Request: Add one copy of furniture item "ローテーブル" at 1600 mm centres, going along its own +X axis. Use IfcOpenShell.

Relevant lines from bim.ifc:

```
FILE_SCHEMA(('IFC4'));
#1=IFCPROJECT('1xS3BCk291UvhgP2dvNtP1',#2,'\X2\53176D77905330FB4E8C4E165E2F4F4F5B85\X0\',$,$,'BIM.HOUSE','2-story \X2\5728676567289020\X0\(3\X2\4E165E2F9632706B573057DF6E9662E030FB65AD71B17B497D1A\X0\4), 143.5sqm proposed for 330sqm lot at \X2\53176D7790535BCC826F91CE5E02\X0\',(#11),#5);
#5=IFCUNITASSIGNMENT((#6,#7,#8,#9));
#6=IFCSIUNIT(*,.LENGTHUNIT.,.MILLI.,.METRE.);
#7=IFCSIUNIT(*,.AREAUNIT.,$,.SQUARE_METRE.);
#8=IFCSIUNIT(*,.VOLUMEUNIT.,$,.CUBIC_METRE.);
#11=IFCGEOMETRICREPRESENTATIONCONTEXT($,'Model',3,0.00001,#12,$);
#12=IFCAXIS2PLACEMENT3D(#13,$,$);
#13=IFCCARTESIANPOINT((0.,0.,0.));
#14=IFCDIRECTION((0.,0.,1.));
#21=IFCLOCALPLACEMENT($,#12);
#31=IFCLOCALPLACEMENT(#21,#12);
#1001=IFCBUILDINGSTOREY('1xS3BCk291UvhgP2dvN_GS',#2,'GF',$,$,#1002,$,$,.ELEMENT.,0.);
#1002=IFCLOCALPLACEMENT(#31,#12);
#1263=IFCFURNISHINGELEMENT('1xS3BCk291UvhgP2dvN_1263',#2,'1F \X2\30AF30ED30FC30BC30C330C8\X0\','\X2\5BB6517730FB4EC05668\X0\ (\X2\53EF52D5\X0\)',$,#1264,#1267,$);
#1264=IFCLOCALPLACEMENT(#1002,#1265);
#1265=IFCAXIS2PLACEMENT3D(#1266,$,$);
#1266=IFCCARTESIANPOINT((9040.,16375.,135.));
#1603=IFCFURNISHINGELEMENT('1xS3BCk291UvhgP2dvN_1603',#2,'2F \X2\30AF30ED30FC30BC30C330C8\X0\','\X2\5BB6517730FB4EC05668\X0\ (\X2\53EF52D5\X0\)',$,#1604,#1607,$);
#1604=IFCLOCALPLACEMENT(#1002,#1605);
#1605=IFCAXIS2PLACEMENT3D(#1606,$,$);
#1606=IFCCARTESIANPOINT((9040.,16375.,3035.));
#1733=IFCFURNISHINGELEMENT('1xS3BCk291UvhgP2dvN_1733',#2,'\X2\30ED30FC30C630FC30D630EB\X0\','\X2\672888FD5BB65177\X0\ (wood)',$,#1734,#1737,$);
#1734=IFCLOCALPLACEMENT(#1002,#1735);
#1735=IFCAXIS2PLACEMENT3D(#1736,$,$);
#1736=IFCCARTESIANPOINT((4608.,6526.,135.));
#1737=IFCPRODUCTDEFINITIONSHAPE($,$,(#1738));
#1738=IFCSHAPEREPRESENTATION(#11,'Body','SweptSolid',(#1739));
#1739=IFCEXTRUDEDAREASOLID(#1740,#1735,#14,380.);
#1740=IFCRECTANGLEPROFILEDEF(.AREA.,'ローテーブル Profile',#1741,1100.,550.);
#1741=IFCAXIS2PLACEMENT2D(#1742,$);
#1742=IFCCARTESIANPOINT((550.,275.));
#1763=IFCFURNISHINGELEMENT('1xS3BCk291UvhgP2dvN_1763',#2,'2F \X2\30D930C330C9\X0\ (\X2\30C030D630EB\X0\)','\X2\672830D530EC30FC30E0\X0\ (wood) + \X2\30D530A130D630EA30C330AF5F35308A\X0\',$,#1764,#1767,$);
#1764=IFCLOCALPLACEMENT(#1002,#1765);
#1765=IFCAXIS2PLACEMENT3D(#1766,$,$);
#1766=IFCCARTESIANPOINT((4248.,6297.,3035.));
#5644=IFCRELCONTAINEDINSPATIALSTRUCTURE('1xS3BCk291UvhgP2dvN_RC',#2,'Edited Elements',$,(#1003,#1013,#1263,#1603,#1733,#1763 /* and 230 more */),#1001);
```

```python
import ifcopenshell
import ifcopenshell.api.geometry
import ifcopenshell.api.root
import ifcopenshell.util.element
import ifcopenshell.util.placement

model = ifcopenshell.open("bim.ifc")


def reuse_history(source, copy):
    """copy_class also copies each property set's owner history, people and application; keep the originals."""
    for rel in copy.IsDefinedBy:
        if rel.is_a("IfcRelDefinesByProperties") and (history := rel.RelatingPropertyDefinition.OwnerHistory):
            rel.RelatingPropertyDefinition.OwnerHistory = source.OwnerHistory
            ifcopenshell.util.element.remove_deep2(model, history)


source = model.by_guid("1xS3BCk291UvhgP2dvN_1733")
base = ifcopenshell.util.placement.get_local_placement(source.ObjectPlacement)
step = base[:3, 0] * 1600.0

for i in range(1, 2):
    copy = ifcopenshell.api.root.copy_class(model, product=source)
    copy.Representation = ifcopenshell.util.element.copy_deep(
        model, source.Representation, exclude=["IfcGeometricRepresentationContext", "IfcRepresentationMap"]
    )
    reuse_history(source, copy)
    matrix = base.copy()
    matrix[:3, 3] += i * step
    print("added at", matrix[:3, 3].round(3) + 0.0)
    ifcopenshell.api.geometry.edit_object_placement(model, product=copy, matrix=matrix, is_si=False)

model.write("bim_rev.ifc")
```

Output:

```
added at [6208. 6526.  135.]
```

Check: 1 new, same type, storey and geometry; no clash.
